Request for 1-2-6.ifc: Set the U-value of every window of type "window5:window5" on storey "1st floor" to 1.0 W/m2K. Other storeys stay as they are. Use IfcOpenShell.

First a look at what the model holds.

```python
import ifcopenshell
import ifcopenshell.util.element

model = ifcopenshell.open("1-2-6.ifc")
print(model.schema)
storey = next(s for s in model.by_type("IfcBuildingStorey") if s.Name == "1st floor")
windows = [e for e in ifcopenshell.util.element.get_decomposition(storey) if e.is_a("IfcWindow")]
seen = {}
for e in windows:
    element_type = ifcopenshell.util.element.get_type(e)
    key = (element_type.Name if element_type != e and element_type else None, ifcopenshell.util.element.get_pset(e, "Pset_WindowCommon", "ThermalTransmittance"))
    seen[key] = seen.get(key, 0) + 1
for (name, value), count in sorted(seen.items(), key=str):
    print(count, "x", name, "|", value)
```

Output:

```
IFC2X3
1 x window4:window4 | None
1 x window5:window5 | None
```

```python
import ifcopenshell
import ifcopenshell.api.pset
import ifcopenshell.util.element

model = ifcopenshell.open("1-2-6.ifc")

storey = next(s for s in model.by_type("IfcBuildingStorey") if s.Name == "1st floor")
windows = [e for e in ifcopenshell.util.element.get_decomposition(storey) if e.is_a("IfcWindow")]

count = 0
for e in windows:
    element_type = ifcopenshell.util.element.get_type(e)
    if element_type in (None, e) or element_type.Name != "window5:window5":
        continue
    # add_pset returns the element's existing set when there is one.
    pset = ifcopenshell.api.pset.add_pset(model, product=e, name="Pset_WindowCommon")
    ifcopenshell.api.pset.edit_pset(model, pset=pset, properties={"ThermalTransmittance": 1.0})
    count += 1

print(count, "windows updated")

model.write("1-2-6_edited.ifc")
```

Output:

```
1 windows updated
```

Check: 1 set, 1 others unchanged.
